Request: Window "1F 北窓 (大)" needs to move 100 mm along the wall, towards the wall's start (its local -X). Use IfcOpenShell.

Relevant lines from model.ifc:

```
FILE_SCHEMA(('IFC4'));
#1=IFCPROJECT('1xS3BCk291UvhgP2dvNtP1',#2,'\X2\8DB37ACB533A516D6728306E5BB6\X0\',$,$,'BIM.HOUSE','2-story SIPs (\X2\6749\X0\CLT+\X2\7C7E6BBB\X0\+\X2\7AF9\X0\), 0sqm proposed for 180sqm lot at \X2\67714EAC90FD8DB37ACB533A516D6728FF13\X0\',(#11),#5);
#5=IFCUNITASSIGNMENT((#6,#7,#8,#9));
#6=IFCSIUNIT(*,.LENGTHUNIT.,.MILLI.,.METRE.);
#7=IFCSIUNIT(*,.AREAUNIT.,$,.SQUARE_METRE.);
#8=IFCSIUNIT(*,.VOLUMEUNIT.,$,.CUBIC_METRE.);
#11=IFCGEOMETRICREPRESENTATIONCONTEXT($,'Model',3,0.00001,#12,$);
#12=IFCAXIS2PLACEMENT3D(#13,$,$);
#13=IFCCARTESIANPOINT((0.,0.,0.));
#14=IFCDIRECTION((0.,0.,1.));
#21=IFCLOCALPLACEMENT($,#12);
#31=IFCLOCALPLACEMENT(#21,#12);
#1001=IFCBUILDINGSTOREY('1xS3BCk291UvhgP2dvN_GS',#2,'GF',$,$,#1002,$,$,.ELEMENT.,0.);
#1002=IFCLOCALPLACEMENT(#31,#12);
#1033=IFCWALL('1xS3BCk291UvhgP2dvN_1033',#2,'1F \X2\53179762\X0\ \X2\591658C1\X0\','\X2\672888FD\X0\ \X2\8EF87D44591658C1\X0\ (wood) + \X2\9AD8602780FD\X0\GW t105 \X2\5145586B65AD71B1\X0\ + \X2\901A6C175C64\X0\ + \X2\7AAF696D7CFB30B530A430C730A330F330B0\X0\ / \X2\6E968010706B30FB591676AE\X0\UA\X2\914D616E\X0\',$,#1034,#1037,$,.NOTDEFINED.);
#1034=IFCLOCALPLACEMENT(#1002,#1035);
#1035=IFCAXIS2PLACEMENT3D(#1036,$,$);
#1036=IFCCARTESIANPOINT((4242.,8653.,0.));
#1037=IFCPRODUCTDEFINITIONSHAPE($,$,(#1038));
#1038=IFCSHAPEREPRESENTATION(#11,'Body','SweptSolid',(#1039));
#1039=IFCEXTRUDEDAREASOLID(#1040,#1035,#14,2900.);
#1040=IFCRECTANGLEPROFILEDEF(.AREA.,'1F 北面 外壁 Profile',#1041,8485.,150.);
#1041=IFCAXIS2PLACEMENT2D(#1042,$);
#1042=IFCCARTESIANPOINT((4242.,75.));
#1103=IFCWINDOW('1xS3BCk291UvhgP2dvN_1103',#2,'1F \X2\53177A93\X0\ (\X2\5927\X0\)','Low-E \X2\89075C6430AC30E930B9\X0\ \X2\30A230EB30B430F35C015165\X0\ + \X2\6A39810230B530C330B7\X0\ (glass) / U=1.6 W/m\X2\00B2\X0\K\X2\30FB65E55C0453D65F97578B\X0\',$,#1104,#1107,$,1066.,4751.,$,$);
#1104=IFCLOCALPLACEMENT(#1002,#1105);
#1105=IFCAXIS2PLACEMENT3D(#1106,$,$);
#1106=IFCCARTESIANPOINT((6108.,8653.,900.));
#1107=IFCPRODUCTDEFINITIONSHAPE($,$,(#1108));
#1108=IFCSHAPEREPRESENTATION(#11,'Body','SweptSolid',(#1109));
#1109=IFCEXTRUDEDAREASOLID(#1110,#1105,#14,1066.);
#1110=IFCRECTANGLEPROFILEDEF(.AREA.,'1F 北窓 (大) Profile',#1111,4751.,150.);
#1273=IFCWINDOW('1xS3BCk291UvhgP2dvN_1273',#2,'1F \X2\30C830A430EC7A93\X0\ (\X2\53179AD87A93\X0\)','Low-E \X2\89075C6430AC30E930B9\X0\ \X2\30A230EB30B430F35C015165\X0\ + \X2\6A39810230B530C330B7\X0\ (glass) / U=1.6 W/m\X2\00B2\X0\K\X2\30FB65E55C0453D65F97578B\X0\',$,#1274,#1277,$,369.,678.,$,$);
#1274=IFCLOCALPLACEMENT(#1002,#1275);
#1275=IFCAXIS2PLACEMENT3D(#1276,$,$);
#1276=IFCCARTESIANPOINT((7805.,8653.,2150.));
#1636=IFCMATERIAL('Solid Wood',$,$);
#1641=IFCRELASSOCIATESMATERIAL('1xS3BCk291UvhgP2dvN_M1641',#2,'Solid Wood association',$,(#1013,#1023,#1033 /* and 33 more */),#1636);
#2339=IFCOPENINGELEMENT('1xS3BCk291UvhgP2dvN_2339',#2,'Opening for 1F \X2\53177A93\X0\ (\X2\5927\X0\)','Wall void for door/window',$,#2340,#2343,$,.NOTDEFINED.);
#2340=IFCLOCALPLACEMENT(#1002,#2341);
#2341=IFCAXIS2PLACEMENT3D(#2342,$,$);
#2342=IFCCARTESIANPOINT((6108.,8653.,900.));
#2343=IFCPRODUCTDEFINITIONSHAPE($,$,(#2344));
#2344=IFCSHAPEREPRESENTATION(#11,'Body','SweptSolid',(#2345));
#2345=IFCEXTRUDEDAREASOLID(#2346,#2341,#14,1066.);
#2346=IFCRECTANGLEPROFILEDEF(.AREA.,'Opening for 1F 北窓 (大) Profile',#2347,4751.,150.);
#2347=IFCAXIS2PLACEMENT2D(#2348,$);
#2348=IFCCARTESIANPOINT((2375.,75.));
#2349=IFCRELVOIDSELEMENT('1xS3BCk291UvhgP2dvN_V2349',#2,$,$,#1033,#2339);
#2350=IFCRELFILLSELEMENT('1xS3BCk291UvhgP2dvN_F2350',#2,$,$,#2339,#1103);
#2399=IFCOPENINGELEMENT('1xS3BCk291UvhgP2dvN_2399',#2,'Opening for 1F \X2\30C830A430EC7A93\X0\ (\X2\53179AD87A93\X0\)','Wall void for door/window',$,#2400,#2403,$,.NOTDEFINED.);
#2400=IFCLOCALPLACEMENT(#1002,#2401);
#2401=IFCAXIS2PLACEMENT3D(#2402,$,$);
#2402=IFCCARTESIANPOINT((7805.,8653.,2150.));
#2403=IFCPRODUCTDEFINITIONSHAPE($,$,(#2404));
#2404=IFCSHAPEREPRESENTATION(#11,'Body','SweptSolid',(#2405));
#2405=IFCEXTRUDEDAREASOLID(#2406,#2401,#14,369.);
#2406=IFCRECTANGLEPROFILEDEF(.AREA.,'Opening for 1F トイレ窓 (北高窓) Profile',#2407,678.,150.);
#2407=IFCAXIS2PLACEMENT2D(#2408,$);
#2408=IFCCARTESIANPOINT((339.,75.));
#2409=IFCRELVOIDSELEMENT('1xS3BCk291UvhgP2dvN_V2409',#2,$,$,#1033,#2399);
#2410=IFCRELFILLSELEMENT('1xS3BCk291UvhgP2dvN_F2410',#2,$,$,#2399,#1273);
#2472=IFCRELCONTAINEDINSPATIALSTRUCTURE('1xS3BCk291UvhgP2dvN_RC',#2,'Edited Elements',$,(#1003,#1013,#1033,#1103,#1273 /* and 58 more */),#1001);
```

```python
import ifcopenshell
import ifcopenshell.api.geometry
import ifcopenshell.util.placement
import ifcopenshell.util.unit

model = ifcopenshell.open("model.ifc")
unit_scale = ifcopenshell.util.unit.calculate_unit_scale(model)

window = model.by_id(1103)
opening = window.FillsVoids[0].RelatingOpeningElement
wall = opening.VoidsElements[0].RelatingBuildingElement

wall_matrix = ifcopenshell.util.placement.get_local_placement(wall.ObjectPlacement)
shift = wall_matrix[:3, 0] * -0.1 / unit_scale
before = ifcopenshell.util.placement.get_local_placement(window.ObjectPlacement)[:3, 3].copy()

# The window is not placed relative to its opening, so move both.
for product in (opening, window):
    matrix = ifcopenshell.util.placement.get_local_placement(product.ObjectPlacement)
    matrix[:3, 3] += shift
    ifcopenshell.api.geometry.edit_object_placement(model, product=product, matrix=matrix, is_si=False)

after = ifcopenshell.util.placement.get_local_placement(window.ObjectPlacement)[:3, 3]
print("window moved by", (after - before).round(3) + 0.0)

model.write("model_edited.ifc")
```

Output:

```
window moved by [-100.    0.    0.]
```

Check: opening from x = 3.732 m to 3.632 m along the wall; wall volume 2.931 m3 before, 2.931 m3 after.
